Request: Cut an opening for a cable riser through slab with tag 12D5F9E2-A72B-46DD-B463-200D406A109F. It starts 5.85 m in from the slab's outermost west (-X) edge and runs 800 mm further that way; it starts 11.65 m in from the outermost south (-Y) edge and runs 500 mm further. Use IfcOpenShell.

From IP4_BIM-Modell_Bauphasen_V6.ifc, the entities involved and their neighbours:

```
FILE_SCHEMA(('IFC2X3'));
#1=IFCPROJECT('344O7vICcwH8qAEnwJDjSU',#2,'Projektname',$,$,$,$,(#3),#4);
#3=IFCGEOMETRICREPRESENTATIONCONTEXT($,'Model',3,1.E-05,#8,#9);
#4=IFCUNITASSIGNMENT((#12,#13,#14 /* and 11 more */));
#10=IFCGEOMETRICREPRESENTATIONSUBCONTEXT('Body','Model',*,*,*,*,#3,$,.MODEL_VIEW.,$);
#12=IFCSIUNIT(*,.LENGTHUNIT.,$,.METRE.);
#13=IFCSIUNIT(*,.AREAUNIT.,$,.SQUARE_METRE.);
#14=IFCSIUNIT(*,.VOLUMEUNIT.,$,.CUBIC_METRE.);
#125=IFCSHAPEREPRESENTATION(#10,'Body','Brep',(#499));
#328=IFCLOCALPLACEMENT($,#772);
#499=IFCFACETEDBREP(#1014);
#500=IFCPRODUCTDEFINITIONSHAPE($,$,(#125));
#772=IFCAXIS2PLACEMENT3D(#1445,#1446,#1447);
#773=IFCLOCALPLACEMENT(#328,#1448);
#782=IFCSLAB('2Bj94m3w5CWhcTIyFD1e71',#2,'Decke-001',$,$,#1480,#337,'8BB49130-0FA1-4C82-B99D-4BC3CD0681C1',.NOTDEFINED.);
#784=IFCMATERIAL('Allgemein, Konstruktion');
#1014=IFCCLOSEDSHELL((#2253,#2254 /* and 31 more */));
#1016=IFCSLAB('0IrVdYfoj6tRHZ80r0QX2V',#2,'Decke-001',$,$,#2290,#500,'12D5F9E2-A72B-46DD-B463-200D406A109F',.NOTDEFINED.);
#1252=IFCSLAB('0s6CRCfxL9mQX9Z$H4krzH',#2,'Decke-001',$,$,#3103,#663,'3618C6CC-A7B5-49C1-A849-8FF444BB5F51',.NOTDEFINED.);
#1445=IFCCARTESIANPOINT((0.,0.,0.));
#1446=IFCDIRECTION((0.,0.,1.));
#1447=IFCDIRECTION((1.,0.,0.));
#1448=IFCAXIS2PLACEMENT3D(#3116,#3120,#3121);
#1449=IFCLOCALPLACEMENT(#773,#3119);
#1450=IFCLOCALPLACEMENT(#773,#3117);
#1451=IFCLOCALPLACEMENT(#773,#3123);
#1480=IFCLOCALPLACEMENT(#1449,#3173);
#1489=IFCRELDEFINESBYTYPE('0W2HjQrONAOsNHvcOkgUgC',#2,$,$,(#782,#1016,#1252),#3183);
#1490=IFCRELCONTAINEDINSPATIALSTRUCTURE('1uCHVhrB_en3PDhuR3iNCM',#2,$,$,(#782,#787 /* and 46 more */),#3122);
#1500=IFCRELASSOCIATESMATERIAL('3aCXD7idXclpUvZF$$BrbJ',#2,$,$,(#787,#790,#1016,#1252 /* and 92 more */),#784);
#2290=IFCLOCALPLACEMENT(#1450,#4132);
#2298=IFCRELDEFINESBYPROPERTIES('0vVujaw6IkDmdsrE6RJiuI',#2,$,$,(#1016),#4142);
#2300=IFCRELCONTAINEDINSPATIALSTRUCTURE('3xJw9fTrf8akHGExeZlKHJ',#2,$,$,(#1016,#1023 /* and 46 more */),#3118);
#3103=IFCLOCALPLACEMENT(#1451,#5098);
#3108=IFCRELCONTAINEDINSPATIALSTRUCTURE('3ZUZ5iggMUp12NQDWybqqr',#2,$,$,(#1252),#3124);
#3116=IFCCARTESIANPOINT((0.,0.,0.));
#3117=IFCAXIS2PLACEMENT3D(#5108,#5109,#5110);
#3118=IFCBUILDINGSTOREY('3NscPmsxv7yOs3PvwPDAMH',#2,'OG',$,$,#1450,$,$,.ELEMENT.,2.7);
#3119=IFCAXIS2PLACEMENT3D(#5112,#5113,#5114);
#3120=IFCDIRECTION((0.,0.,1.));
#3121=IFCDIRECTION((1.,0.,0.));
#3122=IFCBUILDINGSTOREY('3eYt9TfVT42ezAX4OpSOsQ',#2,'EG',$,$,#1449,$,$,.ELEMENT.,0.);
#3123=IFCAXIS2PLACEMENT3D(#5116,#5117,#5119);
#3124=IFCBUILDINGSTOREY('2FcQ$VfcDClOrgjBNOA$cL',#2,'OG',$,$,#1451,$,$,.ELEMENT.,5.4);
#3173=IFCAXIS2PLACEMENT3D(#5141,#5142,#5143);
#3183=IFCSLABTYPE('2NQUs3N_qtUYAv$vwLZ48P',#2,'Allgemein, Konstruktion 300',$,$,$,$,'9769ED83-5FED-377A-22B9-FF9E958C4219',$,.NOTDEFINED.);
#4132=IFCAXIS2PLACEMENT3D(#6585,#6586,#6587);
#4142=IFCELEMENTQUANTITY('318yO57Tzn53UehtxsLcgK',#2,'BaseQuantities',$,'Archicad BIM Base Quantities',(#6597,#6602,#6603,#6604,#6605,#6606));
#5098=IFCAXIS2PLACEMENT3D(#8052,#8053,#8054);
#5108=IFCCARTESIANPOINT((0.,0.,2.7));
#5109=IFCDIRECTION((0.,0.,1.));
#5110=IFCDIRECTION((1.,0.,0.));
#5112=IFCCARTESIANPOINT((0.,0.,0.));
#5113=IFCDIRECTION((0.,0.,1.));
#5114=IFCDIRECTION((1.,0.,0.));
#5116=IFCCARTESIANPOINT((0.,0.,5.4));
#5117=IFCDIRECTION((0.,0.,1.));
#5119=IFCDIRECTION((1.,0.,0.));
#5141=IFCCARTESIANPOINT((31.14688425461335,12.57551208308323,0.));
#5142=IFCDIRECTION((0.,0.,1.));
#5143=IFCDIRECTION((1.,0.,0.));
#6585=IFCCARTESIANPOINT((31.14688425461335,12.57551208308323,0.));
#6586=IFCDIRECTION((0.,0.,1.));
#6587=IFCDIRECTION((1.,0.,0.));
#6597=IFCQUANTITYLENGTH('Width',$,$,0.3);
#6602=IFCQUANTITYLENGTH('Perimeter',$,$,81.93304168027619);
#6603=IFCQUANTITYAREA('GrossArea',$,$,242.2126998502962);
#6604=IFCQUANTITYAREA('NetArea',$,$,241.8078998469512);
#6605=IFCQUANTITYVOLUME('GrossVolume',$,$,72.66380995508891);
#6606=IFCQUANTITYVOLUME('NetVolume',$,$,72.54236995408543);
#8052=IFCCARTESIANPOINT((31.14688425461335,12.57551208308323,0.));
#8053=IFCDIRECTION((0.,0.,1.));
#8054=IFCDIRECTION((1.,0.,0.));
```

```python
import numpy as np
import ifcopenshell
import ifcopenshell.api.feature
import ifcopenshell.api.geometry
import ifcopenshell.api.pset
import ifcopenshell.api.root
import ifcopenshell.geom
import ifcopenshell.util.element
import ifcopenshell.util.placement
import ifcopenshell.util.representation
import ifcopenshell.util.shape
import ifcopenshell.util.unit

model = ifcopenshell.open("IP4_BIM-Modell_Bauphasen_V6.ifc")
unit_scale = ifcopenshell.util.unit.calculate_unit_scale(model)
area_scale = ifcopenshell.util.unit.calculate_unit_scale(model, "AREAUNIT")
volume_scale = ifcopenshell.util.unit.calculate_unit_scale(model, "VOLUMEUNIT")
settings = ifcopenshell.geom.settings()


def volume(element):
    """Net volume in cubic metres, openings subtracted."""
    shape = ifcopenshell.geom.create_shape(settings, element)
    return ifcopenshell.util.shape.get_volume(shape.geometry)


slab = model.by_id(1016)
before = volume(slab)

# Extent in the slab's own axes, in metres. The edges named are its -X and -Y sides.
slab_shape = ifcopenshell.geom.create_shape(settings, slab)
vertices = ifcopenshell.util.shape.get_vertices(slab_shape.geometry)
x_min, y_min, bottom = vertices.min(axis=0)
top = vertices[:, 2].max()

opening = ifcopenshell.api.root.create_entity(model, ifc_class="IfcOpeningElement", name="Cable riser opening")
context = ifcopenshell.util.representation.get_context(model, "Model", "Body", "MODEL_VIEW")
width, depth = 0.8, 0.5
outline = [(0.0, 0.0), (width, 0.0), (width, depth), (0.0, depth), (0.0, 0.0)]
# Overshoot both faces by 50 mm so the cut is clean.
shape = ifcopenshell.api.geometry.add_slab_representation(
    model, context=context, depth=top - bottom + 0.1, polyline=outline
)
ifcopenshell.api.geometry.assign_representation(model, product=opening, representation=shape)

matrix = ifcopenshell.util.placement.get_local_placement(slab.ObjectPlacement)
matrix[:, 3] = matrix @ np.append(np.array([x_min + 5.85, y_min + 11.65, bottom - 0.05]) / unit_scale, 1.0)
ifcopenshell.api.geometry.edit_object_placement(model, product=opening, matrix=matrix, is_si=False)
ifcopenshell.api.feature.add_feature(model, feature=opening, element=slab)

after = volume(slab)

# Update the slab's stored quantities.
qto = model.by_id(ifcopenshell.util.element.get_pset(slab, "BaseQuantities", should_inherit=False)["id"])
ifcopenshell.api.pset.edit_qto(model, qto=qto, properties={
    "NetArea": after / (top - bottom) / area_scale,
    "NetVolume": after / volume_scale,
})

print(f"slab volume {before:.3f} -> {after:.3f} m3")

model.write("IP4_BIM-Modell_Bauphasen_V6-out.ifc")
```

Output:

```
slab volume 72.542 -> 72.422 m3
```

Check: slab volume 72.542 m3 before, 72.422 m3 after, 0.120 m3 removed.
